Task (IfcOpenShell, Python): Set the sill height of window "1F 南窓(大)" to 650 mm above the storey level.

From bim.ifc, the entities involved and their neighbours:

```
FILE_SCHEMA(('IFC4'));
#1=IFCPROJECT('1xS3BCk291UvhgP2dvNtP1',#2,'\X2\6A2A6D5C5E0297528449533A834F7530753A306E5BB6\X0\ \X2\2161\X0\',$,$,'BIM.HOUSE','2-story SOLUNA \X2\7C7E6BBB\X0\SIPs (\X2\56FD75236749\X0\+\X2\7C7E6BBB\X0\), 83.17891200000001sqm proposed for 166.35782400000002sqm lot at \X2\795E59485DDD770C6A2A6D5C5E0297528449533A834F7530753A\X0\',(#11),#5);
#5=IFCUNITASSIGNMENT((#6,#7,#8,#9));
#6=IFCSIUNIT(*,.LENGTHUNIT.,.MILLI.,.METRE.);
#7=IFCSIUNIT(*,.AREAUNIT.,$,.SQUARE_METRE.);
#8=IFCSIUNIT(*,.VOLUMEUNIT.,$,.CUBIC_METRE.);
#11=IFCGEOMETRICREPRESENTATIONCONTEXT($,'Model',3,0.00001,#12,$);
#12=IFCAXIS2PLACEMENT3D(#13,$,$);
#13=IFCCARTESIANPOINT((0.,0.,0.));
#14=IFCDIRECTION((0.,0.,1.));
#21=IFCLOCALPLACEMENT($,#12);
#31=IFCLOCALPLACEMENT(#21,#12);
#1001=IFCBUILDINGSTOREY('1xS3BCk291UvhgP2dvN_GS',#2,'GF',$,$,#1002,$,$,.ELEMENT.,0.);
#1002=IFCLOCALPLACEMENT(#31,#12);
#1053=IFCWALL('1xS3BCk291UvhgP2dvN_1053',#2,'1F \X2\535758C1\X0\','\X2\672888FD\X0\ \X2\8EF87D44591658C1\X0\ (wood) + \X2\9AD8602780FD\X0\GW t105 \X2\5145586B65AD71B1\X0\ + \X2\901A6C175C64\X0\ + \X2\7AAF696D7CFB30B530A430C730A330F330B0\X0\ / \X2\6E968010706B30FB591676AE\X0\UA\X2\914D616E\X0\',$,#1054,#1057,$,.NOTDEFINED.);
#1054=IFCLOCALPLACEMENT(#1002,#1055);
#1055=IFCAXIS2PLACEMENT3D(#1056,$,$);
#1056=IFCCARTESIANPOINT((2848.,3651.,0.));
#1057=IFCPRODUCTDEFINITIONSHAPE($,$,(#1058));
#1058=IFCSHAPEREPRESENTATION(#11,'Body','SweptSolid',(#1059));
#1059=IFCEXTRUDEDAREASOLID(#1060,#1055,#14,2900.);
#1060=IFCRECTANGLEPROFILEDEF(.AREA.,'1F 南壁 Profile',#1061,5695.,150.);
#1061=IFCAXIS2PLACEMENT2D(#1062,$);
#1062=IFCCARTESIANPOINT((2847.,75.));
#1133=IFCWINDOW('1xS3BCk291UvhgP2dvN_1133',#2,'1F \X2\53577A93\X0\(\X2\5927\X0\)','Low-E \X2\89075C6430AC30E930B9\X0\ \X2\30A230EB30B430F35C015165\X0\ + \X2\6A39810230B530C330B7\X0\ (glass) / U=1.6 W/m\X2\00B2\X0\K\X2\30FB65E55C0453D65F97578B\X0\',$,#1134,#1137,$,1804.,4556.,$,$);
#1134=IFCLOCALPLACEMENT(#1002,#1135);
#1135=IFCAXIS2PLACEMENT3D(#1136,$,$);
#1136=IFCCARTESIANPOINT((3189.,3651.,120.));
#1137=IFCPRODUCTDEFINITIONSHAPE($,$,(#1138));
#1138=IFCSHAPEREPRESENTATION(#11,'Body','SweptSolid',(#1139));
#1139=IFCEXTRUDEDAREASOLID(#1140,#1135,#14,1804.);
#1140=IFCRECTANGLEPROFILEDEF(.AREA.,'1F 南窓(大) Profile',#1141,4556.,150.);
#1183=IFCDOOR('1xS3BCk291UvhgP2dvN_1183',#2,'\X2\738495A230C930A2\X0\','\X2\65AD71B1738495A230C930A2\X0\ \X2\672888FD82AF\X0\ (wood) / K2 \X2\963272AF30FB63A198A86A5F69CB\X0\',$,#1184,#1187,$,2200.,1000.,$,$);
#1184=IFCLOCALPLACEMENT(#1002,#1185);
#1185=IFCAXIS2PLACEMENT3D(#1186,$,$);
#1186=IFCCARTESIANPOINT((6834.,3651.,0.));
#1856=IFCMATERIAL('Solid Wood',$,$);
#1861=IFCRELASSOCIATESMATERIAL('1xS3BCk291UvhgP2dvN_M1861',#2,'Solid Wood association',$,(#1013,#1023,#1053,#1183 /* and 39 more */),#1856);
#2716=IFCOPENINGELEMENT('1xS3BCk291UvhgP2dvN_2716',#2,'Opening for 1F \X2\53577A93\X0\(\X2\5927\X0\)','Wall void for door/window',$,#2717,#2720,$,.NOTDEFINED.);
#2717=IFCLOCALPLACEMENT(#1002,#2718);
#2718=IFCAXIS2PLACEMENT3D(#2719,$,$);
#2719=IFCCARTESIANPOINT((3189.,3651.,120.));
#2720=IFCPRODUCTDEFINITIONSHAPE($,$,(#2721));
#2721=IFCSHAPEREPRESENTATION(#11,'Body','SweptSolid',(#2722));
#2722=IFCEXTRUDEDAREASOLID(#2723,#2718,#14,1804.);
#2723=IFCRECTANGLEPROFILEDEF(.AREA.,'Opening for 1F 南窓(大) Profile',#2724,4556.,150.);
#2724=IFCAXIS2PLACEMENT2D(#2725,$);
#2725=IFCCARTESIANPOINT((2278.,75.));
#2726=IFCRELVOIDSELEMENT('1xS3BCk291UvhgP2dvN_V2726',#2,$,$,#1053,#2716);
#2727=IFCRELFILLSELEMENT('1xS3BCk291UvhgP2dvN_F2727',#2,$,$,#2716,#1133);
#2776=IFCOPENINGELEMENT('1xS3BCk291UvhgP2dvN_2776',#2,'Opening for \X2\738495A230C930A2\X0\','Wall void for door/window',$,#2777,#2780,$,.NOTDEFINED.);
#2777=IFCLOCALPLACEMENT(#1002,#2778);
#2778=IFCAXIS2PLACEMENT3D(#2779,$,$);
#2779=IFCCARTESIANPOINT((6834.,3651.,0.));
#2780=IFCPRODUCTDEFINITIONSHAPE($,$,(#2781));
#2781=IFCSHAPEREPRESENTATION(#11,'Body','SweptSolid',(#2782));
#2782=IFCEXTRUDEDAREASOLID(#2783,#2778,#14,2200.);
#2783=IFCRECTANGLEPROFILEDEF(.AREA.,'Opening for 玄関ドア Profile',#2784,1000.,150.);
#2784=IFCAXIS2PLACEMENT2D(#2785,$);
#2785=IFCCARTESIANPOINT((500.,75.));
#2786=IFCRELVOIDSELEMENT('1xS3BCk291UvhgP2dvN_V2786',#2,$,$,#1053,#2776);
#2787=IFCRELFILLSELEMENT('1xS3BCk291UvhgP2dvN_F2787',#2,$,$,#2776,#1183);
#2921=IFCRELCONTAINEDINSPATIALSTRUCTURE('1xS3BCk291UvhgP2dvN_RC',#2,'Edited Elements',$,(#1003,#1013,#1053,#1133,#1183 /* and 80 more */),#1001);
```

```python
import numpy as np
import ifcopenshell
import ifcopenshell.api.geometry
import ifcopenshell.geom
import ifcopenshell.util.element
import ifcopenshell.util.placement
import ifcopenshell.util.shape
import ifcopenshell.util.unit

model = ifcopenshell.open("bim.ifc")
unit_scale = ifcopenshell.util.unit.calculate_unit_scale(model)

window = model.by_guid("1xS3BCk291UvhgP2dvN_1133")
opening = window.FillsVoids[0].RelatingOpeningElement
storey = ifcopenshell.util.element.get_container(window, ifc_class="IfcBuildingStorey")
level = ifcopenshell.util.placement.get_local_placement(storey.ObjectPlacement)[2, 3]

# The opening's origin need not be at the sill, so measure its lowest point.
shape = ifcopenshell.geom.create_shape(ifcopenshell.geom.settings(), opening)
bottom = ifcopenshell.util.shape.get_shape_bottom_elevation(shape, shape.geometry) / unit_scale
dz = level + 650.0 - bottom

shift = np.array([0.0, 0.0, dz])
# The window is not placed relative to its opening, so move both.
for product in (opening, window):
    matrix = ifcopenshell.util.placement.get_local_placement(product.ObjectPlacement)
    matrix[:3, 3] += shift
    ifcopenshell.api.geometry.edit_object_placement(model, product=product, matrix=matrix, is_si=False)

print(f"moved by {dz * unit_scale:+.3f} m")

model.write("bim_edited.ifc")
```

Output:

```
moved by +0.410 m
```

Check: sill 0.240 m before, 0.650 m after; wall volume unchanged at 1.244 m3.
